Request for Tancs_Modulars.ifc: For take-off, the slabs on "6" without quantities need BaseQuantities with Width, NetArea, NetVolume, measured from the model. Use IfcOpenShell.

First a look at what the model holds.

```python
import ifcopenshell
import ifcopenshell.util.element
import ifcopenshell.util.unit

model = ifcopenshell.open("Tancs_Modulars.ifc")
print(model.schema)
for unit_type in ("LENGTHUNIT", "AREAUNIT", "VOLUMEUNIT"):
    print(unit_type, ifcopenshell.util.unit.calculate_unit_scale(model, unit_type))
storey = next(s for s in model.by_type("IfcBuildingStorey") if s.Name == "6")
slabs = [e for e in ifcopenshell.util.element.get_decomposition(storey) if e.is_a("IfcSlab")]
for e in sorted(slabs, key=lambda e: e.id()):
    print(e.id(), e.is_a(), e.Name, list(ifcopenshell.util.element.get_psets(e, qtos_only=True)), sep=" | ")
```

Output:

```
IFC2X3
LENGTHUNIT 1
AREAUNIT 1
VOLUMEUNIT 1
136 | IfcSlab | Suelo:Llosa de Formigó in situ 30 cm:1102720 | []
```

```python
import ifcopenshell
import ifcopenshell.api.pset
import ifcopenshell.geom
import ifcopenshell.util.element
import ifcopenshell.util.shape
import ifcopenshell.util.unit

model = ifcopenshell.open("Tancs_Modulars.ifc")
unit_scale = ifcopenshell.util.unit.calculate_unit_scale(model)
area_scale = ifcopenshell.util.unit.calculate_unit_scale(model, "AREAUNIT")
volume_scale = ifcopenshell.util.unit.calculate_unit_scale(model, "VOLUMEUNIT")
settings = ifcopenshell.geom.settings()

storey = next(s for s in model.by_type("IfcBuildingStorey") if s.Name == "6")
slabs = [e for e in ifcopenshell.util.element.get_decomposition(storey) if e.is_a("IfcSlab")]

for e in sorted(slabs, key=lambda e: e.id()):
    if ifcopenshell.util.element.get_psets(e, qtos_only=True, should_inherit=False):
        continue
    # Geometry comes back in metres, in the element's own axes.
    shape = ifcopenshell.geom.create_shape(settings, e)
    values = {
        "Width": ifcopenshell.util.shape.get_z(shape.geometry) / unit_scale,
        "NetArea": ifcopenshell.util.shape.get_footprint_area(shape.geometry) / area_scale,
        "NetVolume": ifcopenshell.util.shape.get_volume(shape.geometry) / volume_scale,
    }
    qto = ifcopenshell.api.pset.add_qto(model, product=e, name="BaseQuantities")
    ifcopenshell.api.pset.edit_qto(model, qto=qto, properties=values)
    print(e.id(), {k: round(v, 3) for k, v in values.items()})

model.write("Tancs_Modulars_edited.ifc")
```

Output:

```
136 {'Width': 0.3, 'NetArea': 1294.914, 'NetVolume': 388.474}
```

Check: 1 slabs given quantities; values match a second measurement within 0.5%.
